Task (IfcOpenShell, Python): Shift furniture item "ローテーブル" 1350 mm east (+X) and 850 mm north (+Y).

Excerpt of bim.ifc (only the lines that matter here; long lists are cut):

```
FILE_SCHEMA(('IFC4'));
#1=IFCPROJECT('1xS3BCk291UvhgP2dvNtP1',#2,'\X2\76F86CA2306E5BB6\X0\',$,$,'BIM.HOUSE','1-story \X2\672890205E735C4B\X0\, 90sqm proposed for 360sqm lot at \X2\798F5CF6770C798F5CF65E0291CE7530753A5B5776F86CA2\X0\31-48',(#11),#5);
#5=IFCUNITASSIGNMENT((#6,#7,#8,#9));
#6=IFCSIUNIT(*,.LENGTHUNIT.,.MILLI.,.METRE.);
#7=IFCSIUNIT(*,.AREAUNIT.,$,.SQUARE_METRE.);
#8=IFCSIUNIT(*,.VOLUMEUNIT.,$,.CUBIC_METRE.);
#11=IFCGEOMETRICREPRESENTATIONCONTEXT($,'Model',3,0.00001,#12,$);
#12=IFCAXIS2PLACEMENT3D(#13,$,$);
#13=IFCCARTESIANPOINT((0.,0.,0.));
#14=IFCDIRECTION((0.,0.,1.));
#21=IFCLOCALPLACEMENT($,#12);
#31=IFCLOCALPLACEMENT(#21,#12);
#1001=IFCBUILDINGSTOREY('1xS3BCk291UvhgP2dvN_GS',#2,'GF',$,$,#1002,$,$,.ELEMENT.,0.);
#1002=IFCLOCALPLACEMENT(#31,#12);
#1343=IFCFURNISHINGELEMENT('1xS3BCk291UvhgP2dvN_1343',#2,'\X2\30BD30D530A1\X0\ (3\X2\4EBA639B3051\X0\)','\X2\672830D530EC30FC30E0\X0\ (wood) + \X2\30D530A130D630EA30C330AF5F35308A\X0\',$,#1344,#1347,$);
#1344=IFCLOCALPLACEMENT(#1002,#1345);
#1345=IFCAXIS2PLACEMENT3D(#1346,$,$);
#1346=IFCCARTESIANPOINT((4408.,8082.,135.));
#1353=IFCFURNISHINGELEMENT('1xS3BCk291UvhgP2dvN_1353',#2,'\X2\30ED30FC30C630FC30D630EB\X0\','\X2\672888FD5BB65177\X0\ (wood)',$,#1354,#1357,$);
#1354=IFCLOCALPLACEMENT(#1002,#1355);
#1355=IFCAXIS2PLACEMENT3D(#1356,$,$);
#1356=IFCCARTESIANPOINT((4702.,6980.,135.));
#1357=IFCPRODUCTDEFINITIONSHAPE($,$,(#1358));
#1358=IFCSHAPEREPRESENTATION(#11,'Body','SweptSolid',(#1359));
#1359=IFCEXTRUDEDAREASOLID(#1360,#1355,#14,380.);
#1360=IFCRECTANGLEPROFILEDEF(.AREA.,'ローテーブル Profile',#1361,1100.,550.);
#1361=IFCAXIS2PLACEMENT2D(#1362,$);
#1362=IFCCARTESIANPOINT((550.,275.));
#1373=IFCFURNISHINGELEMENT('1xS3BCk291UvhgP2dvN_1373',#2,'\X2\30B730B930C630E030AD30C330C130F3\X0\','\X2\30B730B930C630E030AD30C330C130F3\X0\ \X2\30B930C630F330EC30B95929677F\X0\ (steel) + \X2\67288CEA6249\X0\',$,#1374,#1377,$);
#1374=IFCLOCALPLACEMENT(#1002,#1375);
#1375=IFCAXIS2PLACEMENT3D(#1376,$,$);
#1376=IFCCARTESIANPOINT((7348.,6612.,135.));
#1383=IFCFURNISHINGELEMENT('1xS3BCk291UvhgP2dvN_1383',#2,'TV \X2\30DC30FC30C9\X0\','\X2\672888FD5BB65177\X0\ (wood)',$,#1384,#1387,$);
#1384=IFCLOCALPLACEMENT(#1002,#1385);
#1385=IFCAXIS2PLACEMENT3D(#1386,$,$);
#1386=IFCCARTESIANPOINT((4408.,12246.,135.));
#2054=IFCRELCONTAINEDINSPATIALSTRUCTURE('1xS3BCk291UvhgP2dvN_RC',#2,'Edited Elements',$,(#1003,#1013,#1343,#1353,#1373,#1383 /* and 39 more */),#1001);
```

```python
import ifcopenshell
import ifcopenshell.api.geometry
import ifcopenshell.util.placement

model = ifcopenshell.open("bim.ifc")

item = model.by_guid("1xS3BCk291UvhgP2dvN_1353")
matrix = ifcopenshell.util.placement.get_local_placement(item.ObjectPlacement)
matrix[0, 3] += 1350.0
matrix[1, 3] += 850.0
ifcopenshell.api.geometry.edit_object_placement(model, product=item, matrix=matrix, is_si=False)

print(ifcopenshell.util.placement.get_local_placement(item.ObjectPlacement).round(3) + 0.0)

model.write("bim_v2.ifc")
```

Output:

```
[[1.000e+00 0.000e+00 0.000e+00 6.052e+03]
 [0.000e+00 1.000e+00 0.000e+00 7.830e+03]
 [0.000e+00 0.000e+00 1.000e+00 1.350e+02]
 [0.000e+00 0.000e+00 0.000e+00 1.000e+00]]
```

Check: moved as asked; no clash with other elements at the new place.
